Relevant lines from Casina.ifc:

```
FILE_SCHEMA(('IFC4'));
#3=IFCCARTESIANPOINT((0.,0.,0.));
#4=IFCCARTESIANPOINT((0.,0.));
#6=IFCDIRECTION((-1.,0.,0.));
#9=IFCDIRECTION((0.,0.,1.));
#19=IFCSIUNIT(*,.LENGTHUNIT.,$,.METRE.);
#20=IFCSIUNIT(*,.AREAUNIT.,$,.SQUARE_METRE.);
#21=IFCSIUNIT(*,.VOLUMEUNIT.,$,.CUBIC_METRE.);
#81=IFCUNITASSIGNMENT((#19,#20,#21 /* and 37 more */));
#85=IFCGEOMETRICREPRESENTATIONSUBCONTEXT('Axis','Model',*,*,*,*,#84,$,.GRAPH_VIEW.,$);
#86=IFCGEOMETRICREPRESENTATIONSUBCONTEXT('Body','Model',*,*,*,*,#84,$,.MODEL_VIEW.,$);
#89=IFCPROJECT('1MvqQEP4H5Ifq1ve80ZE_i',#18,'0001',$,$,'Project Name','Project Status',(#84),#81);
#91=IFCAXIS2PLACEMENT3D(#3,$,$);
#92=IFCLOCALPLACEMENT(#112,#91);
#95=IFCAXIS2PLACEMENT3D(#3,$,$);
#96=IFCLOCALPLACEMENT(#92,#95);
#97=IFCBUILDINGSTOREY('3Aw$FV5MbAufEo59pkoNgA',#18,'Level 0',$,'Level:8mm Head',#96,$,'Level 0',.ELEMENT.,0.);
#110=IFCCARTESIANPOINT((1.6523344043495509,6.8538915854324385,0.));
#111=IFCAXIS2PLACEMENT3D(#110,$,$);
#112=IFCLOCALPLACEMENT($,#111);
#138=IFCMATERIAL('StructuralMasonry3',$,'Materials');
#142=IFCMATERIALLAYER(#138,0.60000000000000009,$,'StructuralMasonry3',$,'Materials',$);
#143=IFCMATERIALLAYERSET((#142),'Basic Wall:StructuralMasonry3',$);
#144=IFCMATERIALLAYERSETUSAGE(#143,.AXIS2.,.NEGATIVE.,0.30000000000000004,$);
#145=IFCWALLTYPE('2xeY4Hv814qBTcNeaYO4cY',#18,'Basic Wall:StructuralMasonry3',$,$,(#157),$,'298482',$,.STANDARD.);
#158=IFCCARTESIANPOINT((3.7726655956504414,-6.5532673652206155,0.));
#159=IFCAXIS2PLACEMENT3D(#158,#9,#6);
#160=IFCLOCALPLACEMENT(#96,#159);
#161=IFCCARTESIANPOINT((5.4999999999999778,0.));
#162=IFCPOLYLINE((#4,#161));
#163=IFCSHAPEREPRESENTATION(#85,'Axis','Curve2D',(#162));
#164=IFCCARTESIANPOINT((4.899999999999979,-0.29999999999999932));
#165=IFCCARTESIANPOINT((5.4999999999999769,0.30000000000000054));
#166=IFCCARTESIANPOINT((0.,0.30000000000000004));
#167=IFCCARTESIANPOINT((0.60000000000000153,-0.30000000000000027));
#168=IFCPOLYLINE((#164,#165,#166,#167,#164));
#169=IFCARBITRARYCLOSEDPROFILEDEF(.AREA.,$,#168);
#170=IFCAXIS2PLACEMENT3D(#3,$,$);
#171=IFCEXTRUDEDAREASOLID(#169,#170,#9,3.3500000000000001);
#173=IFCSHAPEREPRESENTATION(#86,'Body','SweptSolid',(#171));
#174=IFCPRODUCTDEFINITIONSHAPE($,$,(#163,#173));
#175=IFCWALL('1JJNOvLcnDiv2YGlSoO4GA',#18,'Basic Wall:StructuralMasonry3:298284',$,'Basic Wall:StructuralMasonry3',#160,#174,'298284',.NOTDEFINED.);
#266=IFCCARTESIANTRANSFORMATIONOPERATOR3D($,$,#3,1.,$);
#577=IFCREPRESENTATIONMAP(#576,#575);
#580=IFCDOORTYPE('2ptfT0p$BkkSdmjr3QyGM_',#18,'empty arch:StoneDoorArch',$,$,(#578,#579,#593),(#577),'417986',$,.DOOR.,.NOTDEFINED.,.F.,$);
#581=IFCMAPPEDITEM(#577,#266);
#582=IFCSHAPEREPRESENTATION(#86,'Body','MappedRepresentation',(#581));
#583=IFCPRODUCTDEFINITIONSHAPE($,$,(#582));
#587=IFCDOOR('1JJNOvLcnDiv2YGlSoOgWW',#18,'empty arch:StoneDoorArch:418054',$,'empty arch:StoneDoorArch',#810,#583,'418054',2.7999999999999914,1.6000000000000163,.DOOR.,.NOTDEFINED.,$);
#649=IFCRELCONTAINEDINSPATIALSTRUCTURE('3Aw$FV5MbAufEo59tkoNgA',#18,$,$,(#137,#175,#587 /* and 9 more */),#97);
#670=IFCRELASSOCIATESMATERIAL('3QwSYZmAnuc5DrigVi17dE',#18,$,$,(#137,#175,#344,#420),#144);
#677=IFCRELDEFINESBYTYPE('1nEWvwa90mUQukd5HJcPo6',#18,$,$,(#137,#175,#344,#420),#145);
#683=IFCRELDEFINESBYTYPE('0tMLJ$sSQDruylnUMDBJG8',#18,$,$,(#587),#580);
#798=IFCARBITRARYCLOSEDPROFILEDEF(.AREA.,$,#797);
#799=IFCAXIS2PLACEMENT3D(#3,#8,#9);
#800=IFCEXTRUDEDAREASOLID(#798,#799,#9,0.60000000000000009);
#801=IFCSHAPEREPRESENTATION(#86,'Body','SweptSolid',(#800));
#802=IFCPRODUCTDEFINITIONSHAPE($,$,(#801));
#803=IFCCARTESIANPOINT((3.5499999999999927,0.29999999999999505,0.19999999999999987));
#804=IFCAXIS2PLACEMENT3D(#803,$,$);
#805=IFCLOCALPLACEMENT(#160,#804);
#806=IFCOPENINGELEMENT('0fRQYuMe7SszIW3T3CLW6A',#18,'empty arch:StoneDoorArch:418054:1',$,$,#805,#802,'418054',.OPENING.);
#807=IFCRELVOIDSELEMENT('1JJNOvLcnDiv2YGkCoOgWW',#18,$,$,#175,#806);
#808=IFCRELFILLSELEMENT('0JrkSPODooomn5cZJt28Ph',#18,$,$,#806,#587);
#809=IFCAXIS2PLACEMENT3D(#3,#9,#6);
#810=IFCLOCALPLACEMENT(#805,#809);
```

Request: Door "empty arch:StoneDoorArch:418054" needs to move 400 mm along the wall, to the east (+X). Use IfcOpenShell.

```python
import ifcopenshell
import ifcopenshell.api.geometry
import ifcopenshell.util.placement
import ifcopenshell.util.unit

model = ifcopenshell.open("Casina.ifc")
unit_scale = ifcopenshell.util.unit.calculate_unit_scale(model)

door = model.by_id(587)
opening = door.FillsVoids[0].RelatingOpeningElement
wall = opening.VoidsElements[0].RelatingBuildingElement

wall_matrix = ifcopenshell.util.placement.get_local_placement(wall.ObjectPlacement)
shift = wall_matrix[:3, 0] * -0.4 / unit_scale
before = ifcopenshell.util.placement.get_local_placement(door.ObjectPlacement)[:3, 3].copy()

# The door is placed relative to its opening, so it follows when the opening moves.
matrix = ifcopenshell.util.placement.get_local_placement(opening.ObjectPlacement)
matrix[:3, 3] += shift
ifcopenshell.api.geometry.edit_object_placement(
    model, product=opening, matrix=matrix, is_si=False, should_transform_children=True
)

after = ifcopenshell.util.placement.get_local_placement(door.ObjectPlacement)[:3, 3]
print("door moved by", (after - before).round(3) + 0.0)

model.write("Casina_v2.ifc")
```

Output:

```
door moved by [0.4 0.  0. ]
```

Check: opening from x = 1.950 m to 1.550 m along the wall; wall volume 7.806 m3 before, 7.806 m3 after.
